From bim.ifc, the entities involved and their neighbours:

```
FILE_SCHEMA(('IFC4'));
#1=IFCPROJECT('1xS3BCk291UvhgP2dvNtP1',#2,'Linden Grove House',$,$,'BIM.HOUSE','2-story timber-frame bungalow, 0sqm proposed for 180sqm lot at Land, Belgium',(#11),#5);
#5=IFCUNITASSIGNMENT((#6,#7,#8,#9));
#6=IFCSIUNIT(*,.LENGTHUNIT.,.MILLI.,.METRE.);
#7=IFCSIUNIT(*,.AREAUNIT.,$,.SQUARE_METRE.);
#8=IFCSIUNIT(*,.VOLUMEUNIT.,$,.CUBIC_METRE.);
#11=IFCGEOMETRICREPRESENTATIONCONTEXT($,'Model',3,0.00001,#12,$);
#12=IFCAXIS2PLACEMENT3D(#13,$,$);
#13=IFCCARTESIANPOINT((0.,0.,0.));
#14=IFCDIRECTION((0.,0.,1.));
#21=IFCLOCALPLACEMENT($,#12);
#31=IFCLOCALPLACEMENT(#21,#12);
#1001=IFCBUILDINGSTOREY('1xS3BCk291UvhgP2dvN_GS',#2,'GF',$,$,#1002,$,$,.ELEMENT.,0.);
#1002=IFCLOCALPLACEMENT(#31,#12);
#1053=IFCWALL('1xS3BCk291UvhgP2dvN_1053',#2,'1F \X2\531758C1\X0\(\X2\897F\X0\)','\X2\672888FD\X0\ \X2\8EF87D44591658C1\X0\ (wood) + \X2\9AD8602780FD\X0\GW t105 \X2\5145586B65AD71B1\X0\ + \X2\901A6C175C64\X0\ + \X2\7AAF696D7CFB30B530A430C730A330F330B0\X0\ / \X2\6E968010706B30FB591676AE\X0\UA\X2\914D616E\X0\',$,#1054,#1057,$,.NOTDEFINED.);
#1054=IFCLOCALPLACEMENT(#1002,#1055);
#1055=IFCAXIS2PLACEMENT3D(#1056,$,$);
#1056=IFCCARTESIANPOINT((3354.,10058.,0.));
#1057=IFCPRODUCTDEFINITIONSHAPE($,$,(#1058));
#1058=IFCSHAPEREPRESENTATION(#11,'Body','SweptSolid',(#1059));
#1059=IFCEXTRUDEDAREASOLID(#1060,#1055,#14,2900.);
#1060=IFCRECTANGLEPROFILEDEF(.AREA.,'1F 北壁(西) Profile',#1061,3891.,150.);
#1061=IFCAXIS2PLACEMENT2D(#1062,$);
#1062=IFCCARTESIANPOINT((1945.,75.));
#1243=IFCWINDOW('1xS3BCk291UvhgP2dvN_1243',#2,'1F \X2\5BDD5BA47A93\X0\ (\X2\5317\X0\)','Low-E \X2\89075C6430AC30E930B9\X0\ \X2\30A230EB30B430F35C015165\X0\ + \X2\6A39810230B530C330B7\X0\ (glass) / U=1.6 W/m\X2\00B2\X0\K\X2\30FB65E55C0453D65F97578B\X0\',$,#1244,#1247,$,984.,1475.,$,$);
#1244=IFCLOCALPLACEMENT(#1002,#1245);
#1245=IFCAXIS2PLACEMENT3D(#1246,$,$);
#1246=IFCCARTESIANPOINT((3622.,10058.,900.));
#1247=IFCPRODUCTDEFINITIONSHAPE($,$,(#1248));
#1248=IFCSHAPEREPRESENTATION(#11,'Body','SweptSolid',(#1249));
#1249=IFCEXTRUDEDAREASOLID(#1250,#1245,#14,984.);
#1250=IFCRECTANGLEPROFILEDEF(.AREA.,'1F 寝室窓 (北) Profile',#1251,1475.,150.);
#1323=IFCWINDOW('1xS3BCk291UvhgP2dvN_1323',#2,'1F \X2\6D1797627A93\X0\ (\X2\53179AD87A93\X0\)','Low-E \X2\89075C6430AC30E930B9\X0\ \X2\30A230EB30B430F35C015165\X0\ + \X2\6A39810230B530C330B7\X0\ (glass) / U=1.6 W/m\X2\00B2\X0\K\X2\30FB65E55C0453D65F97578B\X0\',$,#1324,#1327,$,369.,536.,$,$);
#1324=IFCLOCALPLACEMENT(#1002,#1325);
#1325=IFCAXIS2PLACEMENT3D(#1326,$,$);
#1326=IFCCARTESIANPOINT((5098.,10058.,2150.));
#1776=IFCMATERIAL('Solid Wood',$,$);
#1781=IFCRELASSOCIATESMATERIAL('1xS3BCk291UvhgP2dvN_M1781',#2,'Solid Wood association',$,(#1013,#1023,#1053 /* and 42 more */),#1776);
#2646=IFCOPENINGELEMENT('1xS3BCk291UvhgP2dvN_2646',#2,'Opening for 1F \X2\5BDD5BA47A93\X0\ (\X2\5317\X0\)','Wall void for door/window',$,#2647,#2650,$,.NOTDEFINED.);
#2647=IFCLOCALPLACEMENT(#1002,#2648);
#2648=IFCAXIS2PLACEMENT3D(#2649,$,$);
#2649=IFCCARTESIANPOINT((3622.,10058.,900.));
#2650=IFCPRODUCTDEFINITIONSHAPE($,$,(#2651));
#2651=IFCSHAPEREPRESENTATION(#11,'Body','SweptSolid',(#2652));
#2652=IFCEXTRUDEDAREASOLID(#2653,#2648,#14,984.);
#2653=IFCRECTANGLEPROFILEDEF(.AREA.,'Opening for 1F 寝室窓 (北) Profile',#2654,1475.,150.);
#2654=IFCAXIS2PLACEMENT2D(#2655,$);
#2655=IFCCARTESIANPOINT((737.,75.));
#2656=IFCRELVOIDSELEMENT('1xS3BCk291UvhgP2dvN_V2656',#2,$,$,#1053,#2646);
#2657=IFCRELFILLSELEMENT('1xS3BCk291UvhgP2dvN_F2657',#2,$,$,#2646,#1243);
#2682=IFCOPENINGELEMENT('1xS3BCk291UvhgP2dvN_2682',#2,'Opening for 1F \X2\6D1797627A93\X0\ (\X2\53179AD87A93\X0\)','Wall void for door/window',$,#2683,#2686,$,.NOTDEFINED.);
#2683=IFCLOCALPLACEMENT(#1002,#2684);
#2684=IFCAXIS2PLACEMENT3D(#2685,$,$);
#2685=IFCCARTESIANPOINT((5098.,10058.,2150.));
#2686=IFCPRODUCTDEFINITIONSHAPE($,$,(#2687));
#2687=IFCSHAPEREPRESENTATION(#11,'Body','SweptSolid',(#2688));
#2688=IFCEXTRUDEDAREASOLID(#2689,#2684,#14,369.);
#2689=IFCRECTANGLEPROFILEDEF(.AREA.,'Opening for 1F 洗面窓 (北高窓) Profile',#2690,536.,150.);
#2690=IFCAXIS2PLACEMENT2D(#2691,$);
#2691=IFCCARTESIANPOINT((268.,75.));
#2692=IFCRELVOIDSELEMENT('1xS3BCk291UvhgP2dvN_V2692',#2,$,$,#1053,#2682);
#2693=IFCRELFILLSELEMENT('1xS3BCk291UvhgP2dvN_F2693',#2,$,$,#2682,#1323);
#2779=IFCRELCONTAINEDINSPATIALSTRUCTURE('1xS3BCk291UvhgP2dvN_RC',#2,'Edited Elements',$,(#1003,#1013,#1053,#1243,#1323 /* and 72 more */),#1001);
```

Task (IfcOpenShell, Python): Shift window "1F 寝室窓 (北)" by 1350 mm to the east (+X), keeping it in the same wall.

```python
import ifcopenshell
import ifcopenshell.api.geometry
import ifcopenshell.util.placement

model = ifcopenshell.open("bim.ifc")

window = model.by_guid("1xS3BCk291UvhgP2dvN_1243")
opening = window.FillsVoids[0].RelatingOpeningElement
wall = opening.VoidsElements[0].RelatingBuildingElement

wall_matrix = ifcopenshell.util.placement.get_local_placement(wall.ObjectPlacement)
shift = wall_matrix[:3, 0] * 1350.0
before = ifcopenshell.util.placement.get_local_placement(window.ObjectPlacement)[:3, 3].copy()

# The window is not placed relative to its opening, so move both.
for product in (opening, window):
    matrix = ifcopenshell.util.placement.get_local_placement(product.ObjectPlacement)
    matrix[:3, 3] += shift
    ifcopenshell.api.geometry.edit_object_placement(model, product=product, matrix=matrix, is_si=False)

after = ifcopenshell.util.placement.get_local_placement(window.ObjectPlacement)[:3, 3]
print("window moved by", (after - before).round(3) + 0.0)

model.write("bim_rev.ifc")
```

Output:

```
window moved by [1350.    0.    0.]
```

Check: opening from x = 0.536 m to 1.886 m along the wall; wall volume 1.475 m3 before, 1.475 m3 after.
